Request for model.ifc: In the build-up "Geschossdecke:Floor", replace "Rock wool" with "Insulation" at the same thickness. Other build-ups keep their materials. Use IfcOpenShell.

First a look at what the model holds.

```python
import ifcopenshell
import ifcopenshell.util.element

model = ifcopenshell.open("model.ifc")
print(model.schema)
for layer_set in model.by_type("IfcMaterialLayerSet"):
    if layer_set.LayerSetName == "Geschossdecke:Floor":
        for layer in layer_set.MaterialLayers:
            print(layer.id(), layer.Material and layer.Material.Name, layer.LayerThickness, sep=" | ")
        print(len(ifcopenshell.util.element.get_elements_by_material(model, layer_set)), "elements and types use it")
print(sorted(m.Name for m in model.by_type("IfcMaterial") if m.Name)[:60])
```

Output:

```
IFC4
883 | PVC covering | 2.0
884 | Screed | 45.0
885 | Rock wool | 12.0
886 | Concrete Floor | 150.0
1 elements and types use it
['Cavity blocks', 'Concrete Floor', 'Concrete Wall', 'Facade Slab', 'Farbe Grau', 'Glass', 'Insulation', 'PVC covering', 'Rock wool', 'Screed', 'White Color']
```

```python
import ifcopenshell
import ifcopenshell.api.material

model = ifcopenshell.open("model.ifc")

layer_set = next(s for s in model.by_type("IfcMaterialLayerSet") if s.LayerSetName == "Geschossdecke:Floor")
layer = next(l for l in layer_set.MaterialLayers if l.Material and l.Material.Name == "Rock wool")
material = next(m for m in model.by_type("IfcMaterial") if m.Name == "Insulation")

# Point this one layer at the other material; renaming the old one would change it everywhere.
ifcopenshell.api.material.edit_layer(model, layer=layer, attributes={}, material=material)

print([l.Material.Name if l.Material else None for l in layer_set.MaterialLayers])

model.write("model-out.ifc")
```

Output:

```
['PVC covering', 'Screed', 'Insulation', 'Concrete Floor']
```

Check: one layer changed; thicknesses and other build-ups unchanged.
